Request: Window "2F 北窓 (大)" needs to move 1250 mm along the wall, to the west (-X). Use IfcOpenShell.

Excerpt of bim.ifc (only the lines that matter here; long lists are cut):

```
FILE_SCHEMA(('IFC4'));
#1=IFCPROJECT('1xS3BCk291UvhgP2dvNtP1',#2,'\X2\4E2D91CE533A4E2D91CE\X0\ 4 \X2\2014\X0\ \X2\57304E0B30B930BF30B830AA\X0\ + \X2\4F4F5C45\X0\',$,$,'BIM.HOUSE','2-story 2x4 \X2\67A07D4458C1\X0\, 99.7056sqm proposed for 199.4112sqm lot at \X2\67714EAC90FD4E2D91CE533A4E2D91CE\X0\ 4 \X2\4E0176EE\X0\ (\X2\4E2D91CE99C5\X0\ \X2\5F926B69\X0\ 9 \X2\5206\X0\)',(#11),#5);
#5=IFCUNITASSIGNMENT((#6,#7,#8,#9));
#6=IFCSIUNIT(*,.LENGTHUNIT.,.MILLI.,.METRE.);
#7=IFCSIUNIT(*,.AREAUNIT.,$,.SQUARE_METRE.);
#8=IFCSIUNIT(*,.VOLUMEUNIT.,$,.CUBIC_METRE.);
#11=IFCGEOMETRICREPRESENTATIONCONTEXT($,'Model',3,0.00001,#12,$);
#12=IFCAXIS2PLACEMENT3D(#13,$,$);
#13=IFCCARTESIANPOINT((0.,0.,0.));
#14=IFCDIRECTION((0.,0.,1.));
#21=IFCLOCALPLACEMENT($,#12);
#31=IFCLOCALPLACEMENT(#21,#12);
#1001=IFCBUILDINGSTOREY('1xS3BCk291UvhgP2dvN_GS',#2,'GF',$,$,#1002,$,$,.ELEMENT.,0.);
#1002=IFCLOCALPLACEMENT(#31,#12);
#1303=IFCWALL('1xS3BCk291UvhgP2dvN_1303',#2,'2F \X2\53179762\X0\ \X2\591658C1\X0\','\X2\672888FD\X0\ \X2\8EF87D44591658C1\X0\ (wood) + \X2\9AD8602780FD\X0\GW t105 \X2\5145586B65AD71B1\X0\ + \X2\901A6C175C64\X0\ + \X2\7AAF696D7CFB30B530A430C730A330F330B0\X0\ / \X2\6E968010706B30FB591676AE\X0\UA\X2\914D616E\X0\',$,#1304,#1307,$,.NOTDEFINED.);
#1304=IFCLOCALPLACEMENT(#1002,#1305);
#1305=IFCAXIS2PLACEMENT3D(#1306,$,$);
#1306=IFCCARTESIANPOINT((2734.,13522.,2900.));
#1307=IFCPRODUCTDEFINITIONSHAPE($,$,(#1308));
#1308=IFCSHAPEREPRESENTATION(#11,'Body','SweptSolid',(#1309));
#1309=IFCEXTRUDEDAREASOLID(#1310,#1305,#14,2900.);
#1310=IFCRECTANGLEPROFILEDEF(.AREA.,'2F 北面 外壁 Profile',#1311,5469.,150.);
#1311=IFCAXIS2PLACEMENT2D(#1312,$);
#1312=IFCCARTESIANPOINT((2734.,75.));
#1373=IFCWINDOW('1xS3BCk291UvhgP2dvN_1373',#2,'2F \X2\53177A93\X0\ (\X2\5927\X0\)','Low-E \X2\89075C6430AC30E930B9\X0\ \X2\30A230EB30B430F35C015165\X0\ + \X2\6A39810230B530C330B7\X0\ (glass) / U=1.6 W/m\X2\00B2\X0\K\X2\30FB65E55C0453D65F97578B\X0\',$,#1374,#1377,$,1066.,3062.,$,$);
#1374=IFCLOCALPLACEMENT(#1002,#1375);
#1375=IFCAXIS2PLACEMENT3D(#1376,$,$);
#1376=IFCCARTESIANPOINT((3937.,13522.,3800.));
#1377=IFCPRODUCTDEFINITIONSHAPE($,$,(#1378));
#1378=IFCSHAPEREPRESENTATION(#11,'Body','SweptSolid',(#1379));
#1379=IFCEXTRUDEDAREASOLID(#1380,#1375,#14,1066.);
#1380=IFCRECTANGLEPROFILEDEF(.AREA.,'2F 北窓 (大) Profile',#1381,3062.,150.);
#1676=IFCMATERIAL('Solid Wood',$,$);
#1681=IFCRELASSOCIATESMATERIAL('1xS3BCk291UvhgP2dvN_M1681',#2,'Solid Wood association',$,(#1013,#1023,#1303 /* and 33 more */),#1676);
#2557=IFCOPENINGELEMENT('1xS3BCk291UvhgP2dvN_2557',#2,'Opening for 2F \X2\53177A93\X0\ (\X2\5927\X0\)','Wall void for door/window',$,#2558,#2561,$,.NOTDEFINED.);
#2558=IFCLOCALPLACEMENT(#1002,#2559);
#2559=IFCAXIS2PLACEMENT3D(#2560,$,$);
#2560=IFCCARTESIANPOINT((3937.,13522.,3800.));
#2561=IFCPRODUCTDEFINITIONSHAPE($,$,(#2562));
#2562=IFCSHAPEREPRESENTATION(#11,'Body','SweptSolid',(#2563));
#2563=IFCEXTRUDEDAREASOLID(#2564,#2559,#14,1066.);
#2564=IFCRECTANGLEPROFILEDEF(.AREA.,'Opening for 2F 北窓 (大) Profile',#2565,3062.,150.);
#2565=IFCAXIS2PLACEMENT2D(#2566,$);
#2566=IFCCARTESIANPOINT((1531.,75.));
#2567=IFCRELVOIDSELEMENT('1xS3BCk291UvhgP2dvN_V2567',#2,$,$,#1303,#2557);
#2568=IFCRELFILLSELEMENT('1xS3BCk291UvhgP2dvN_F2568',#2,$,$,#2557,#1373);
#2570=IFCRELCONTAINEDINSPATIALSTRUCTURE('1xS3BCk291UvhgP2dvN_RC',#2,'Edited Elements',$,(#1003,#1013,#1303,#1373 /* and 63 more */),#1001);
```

```python
import ifcopenshell
import ifcopenshell.api.geometry
import ifcopenshell.util.placement

model = ifcopenshell.open("bim.ifc")

window = model.by_guid("1xS3BCk291UvhgP2dvN_1373")
opening = window.FillsVoids[0].RelatingOpeningElement
wall = opening.VoidsElements[0].RelatingBuildingElement

wall_matrix = ifcopenshell.util.placement.get_local_placement(wall.ObjectPlacement)
shift = wall_matrix[:3, 0] * -1250.0
before = ifcopenshell.util.placement.get_local_placement(window.ObjectPlacement)[:3, 3].copy()

# The window is not placed relative to its opening, so move both.
for product in (opening, window):
    matrix = ifcopenshell.util.placement.get_local_placement(product.ObjectPlacement)
    matrix[:3, 3] += shift
    ifcopenshell.api.geometry.edit_object_placement(model, product=product, matrix=matrix, is_si=False)

after = ifcopenshell.util.placement.get_local_placement(window.ObjectPlacement)[:3, 3]
print("window moved by", (after - before).round(3) + 0.0)

model.write("bim_edited.ifc")
```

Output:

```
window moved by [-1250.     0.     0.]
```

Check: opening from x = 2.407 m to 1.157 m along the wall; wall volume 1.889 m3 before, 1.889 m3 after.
